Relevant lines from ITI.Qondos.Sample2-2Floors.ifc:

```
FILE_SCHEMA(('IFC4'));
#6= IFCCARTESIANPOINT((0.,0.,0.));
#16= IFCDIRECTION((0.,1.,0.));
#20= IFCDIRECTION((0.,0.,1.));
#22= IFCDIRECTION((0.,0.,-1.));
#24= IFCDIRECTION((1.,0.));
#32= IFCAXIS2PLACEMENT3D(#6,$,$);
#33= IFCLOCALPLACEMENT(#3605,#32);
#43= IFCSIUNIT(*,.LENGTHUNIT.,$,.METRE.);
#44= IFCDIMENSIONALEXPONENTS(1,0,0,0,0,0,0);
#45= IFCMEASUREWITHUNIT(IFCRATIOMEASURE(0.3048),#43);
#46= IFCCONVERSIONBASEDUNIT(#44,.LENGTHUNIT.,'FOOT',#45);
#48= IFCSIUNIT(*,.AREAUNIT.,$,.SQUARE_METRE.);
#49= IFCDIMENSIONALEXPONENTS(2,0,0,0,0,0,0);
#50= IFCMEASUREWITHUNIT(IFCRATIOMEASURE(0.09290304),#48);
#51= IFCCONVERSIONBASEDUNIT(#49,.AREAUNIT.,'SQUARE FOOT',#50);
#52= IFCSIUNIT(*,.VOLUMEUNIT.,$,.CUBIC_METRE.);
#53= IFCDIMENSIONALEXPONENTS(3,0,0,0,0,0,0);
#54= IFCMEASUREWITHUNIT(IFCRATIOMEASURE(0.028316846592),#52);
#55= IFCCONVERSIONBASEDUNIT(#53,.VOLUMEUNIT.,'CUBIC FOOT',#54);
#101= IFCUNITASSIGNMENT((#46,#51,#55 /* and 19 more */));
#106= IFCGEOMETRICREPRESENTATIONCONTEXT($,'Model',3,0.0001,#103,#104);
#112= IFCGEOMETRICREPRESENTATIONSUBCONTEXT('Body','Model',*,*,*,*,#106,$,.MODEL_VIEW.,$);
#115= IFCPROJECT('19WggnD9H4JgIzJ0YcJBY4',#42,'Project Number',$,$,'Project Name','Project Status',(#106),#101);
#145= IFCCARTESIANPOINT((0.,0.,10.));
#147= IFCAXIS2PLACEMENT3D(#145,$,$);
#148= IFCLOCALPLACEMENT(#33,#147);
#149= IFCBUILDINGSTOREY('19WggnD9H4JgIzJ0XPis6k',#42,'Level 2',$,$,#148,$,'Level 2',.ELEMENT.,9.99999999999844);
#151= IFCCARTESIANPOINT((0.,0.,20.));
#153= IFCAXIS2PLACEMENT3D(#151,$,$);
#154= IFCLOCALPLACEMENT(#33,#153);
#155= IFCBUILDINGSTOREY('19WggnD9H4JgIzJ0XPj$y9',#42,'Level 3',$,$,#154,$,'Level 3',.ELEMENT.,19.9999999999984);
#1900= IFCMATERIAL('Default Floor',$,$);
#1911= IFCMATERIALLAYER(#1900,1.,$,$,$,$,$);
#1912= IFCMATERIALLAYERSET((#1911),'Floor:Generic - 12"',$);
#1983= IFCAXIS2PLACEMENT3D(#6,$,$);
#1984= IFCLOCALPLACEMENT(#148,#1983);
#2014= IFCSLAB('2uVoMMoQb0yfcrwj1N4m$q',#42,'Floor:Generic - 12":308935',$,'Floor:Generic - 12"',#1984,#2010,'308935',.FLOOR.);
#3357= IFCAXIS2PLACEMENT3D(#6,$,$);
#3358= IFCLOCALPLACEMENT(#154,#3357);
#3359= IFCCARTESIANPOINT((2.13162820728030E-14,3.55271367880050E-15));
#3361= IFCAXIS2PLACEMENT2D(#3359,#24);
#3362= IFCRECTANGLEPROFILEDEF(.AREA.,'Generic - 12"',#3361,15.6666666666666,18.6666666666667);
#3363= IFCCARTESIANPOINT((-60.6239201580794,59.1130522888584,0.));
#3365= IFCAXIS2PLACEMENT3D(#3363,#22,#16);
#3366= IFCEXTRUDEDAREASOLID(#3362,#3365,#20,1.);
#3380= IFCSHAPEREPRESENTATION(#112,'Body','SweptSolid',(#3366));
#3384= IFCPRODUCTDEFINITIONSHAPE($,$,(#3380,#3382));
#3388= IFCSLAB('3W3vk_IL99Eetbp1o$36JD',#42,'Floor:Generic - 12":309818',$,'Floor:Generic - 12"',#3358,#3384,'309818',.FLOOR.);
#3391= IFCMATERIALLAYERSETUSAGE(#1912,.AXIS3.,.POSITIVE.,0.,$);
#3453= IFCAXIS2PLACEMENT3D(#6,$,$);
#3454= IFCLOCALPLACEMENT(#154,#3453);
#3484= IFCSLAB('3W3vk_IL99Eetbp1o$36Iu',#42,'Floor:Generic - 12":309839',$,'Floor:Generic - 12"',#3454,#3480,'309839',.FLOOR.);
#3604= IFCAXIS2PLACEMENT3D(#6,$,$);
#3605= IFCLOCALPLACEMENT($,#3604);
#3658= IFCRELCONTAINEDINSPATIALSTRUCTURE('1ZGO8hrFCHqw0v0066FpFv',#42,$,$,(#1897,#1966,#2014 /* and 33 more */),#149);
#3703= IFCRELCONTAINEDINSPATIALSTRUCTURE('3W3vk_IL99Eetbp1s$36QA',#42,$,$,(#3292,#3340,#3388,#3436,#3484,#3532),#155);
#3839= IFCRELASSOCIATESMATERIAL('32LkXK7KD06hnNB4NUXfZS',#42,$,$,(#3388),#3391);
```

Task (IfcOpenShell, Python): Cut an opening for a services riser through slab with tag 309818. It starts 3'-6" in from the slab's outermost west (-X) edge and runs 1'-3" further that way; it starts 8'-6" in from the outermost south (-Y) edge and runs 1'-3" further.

```python
import numpy as np
import ifcopenshell
import ifcopenshell.api.feature
import ifcopenshell.api.geometry
import ifcopenshell.api.root
import ifcopenshell.geom
import ifcopenshell.util.placement
import ifcopenshell.util.representation
import ifcopenshell.util.shape
import ifcopenshell.util.unit

model = ifcopenshell.open("ITI.Qondos.Sample2-2Floors.ifc")
unit_scale = ifcopenshell.util.unit.calculate_unit_scale(model)
settings = ifcopenshell.geom.settings()


def volume(element):
    """Net volume in cubic metres, openings subtracted."""
    shape = ifcopenshell.geom.create_shape(settings, element)
    return ifcopenshell.util.shape.get_volume(shape.geometry)


slab = model.by_guid("3W3vk_IL99Eetbp1o$36JD")
before = volume(slab)

# Extent in the slab's own axes, in metres. The edges named are its -X and -Y sides.
slab_shape = ifcopenshell.geom.create_shape(settings, slab)
vertices = ifcopenshell.util.shape.get_vertices(slab_shape.geometry)
x_min, y_min, bottom = vertices.min(axis=0)
top = vertices[:, 2].max()

opening = ifcopenshell.api.root.create_entity(model, ifc_class="IfcOpeningElement", name="Services riser opening", predefined_type="OPENING")
context = ifcopenshell.util.representation.get_context(model, "Model", "Body", "MODEL_VIEW")
width, depth = 0.381, 0.381
outline = [(0.0, 0.0), (width, 0.0), (width, depth), (0.0, depth), (0.0, 0.0)]
# Overshoot both faces by 50 mm so the cut is clean.
shape = ifcopenshell.api.geometry.add_slab_representation(
    model, context=context, depth=top - bottom + 0.1, polyline=outline
)
ifcopenshell.api.geometry.assign_representation(model, product=opening, representation=shape)

matrix = ifcopenshell.util.placement.get_local_placement(slab.ObjectPlacement)
matrix[:, 3] = matrix @ np.append(np.array([x_min + 1.0668, y_min + 2.5908, bottom - 0.05]) / unit_scale, 1.0)
ifcopenshell.api.geometry.edit_object_placement(model, product=opening, matrix=matrix, is_si=False)
ifcopenshell.api.feature.add_feature(model, feature=opening, element=slab)

after = volume(slab)

print(f"slab volume {before:.3f} -> {after:.3f} m3")

model.write("ITI.Qondos.Sample2-2Floors_updated.ifc")
```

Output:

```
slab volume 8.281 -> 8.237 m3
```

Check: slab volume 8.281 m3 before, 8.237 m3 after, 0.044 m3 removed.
